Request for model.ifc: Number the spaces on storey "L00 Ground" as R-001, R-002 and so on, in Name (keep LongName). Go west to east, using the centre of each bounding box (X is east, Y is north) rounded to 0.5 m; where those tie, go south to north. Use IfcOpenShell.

First a look at what the model holds.

```python
import ifcopenshell
import ifcopenshell.util.element
import ifcopenshell.util.placement

model = ifcopenshell.open("model.ifc")
print(model.schema)
storey = next(s for s in model.by_type("IfcBuildingStorey") if s.Name == "L00 Ground")
spaces = [e for e in ifcopenshell.util.element.get_decomposition(storey) if e.is_a("IfcSpace")]
for e in sorted(spaces, key=lambda e: e.id()):
    origin = ifcopenshell.util.placement.get_local_placement(e.ObjectPlacement)[:3, 3]
    print(e.id(), e.Name, e.LongName, origin.round(2) + 0.0, sep=" | ")
```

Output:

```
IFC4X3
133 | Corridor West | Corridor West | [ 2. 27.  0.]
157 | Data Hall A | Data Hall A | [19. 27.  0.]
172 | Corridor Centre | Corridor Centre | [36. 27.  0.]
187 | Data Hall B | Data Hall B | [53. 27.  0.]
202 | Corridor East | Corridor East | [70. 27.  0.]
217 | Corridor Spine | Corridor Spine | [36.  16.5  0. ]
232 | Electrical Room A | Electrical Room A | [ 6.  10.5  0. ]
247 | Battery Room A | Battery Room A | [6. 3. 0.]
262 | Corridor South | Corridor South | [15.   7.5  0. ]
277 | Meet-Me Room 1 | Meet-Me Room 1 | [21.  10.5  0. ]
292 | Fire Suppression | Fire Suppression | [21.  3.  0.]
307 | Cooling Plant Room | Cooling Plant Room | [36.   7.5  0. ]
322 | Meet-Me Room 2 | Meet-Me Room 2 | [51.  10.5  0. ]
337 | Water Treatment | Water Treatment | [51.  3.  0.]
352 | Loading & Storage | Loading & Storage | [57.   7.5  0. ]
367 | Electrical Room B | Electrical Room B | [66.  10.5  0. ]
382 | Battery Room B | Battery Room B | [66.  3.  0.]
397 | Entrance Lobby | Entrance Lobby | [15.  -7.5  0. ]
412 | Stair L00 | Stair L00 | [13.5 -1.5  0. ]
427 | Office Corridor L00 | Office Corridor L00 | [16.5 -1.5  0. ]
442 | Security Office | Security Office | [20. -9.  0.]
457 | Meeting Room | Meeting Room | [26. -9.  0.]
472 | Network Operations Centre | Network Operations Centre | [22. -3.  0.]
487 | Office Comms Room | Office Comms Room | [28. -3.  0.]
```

```python
import ifcopenshell
import ifcopenshell.geom
import ifcopenshell.util.element
import ifcopenshell.util.shape

model = ifcopenshell.open("model.ifc")
settings = ifcopenshell.geom.settings()
settings.set("use-world-coords", True)


def centre(element):
    shape = ifcopenshell.geom.create_shape(settings, element)
    return ifcopenshell.util.shape.get_bbox_centroid(shape.geometry)


storey = next(s for s in model.by_type("IfcBuildingStorey") if s.Name == "L00 Ground")
spaces = [e for e in ifcopenshell.util.element.get_decomposition(storey) if e.is_a("IfcSpace")]

# Insertion points can sit at a corner or the storey origin, so sort by the geometry (in metres).
centres = {e: centre(e) for e in spaces}
spaces.sort(key=lambda e: (round(centres[e][0] / 0.5), centres[e][1]))

for i, e in enumerate(spaces, start=1):
    number = f"R-0{i:02d}"
    e.Name = number
    print(e.id(), number)

model.write("model_rev.ifc")
```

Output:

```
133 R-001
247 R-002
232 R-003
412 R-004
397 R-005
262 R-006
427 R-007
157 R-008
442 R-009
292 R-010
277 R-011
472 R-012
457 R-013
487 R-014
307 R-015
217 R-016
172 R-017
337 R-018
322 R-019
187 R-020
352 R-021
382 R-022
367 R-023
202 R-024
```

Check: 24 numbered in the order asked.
